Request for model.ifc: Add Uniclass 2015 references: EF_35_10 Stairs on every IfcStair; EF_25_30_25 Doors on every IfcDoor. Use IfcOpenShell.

First a look at what the model holds.

```python
import ifcopenshell

model = ifcopenshell.open("model.ifc")
print(model.schema)
print("classifications:", [c.Name for c in model.by_type("IfcClassification")])
for ifc_class in ("IfcDoor", "IfcRoof", "IfcStair", "IfcWall", "IfcWindow"):
    print(ifc_class, len(model.by_type(ifc_class)))
```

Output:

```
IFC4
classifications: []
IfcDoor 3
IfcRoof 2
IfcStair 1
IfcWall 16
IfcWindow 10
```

```python
import ifcopenshell
import ifcopenshell.api.classification

model = ifcopenshell.open("model.ifc")

system = ifcopenshell.api.classification.add_classification(model, classification="Uniclass 2015")

codes = {
    "IfcStair": ("EF_35_10", "Stairs"),
    "IfcDoor": ("EF_25_30_25", "Doors"),
}
for ifc_class, (code, name) in codes.items():
    products = model.by_type(ifc_class)
    ifcopenshell.api.classification.add_reference(
        model, products=products, classification=system, identification=code, name=name
    )
    print(code, len(products))

model.write("model_updated.ifc")
```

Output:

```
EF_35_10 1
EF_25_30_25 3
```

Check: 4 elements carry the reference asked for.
